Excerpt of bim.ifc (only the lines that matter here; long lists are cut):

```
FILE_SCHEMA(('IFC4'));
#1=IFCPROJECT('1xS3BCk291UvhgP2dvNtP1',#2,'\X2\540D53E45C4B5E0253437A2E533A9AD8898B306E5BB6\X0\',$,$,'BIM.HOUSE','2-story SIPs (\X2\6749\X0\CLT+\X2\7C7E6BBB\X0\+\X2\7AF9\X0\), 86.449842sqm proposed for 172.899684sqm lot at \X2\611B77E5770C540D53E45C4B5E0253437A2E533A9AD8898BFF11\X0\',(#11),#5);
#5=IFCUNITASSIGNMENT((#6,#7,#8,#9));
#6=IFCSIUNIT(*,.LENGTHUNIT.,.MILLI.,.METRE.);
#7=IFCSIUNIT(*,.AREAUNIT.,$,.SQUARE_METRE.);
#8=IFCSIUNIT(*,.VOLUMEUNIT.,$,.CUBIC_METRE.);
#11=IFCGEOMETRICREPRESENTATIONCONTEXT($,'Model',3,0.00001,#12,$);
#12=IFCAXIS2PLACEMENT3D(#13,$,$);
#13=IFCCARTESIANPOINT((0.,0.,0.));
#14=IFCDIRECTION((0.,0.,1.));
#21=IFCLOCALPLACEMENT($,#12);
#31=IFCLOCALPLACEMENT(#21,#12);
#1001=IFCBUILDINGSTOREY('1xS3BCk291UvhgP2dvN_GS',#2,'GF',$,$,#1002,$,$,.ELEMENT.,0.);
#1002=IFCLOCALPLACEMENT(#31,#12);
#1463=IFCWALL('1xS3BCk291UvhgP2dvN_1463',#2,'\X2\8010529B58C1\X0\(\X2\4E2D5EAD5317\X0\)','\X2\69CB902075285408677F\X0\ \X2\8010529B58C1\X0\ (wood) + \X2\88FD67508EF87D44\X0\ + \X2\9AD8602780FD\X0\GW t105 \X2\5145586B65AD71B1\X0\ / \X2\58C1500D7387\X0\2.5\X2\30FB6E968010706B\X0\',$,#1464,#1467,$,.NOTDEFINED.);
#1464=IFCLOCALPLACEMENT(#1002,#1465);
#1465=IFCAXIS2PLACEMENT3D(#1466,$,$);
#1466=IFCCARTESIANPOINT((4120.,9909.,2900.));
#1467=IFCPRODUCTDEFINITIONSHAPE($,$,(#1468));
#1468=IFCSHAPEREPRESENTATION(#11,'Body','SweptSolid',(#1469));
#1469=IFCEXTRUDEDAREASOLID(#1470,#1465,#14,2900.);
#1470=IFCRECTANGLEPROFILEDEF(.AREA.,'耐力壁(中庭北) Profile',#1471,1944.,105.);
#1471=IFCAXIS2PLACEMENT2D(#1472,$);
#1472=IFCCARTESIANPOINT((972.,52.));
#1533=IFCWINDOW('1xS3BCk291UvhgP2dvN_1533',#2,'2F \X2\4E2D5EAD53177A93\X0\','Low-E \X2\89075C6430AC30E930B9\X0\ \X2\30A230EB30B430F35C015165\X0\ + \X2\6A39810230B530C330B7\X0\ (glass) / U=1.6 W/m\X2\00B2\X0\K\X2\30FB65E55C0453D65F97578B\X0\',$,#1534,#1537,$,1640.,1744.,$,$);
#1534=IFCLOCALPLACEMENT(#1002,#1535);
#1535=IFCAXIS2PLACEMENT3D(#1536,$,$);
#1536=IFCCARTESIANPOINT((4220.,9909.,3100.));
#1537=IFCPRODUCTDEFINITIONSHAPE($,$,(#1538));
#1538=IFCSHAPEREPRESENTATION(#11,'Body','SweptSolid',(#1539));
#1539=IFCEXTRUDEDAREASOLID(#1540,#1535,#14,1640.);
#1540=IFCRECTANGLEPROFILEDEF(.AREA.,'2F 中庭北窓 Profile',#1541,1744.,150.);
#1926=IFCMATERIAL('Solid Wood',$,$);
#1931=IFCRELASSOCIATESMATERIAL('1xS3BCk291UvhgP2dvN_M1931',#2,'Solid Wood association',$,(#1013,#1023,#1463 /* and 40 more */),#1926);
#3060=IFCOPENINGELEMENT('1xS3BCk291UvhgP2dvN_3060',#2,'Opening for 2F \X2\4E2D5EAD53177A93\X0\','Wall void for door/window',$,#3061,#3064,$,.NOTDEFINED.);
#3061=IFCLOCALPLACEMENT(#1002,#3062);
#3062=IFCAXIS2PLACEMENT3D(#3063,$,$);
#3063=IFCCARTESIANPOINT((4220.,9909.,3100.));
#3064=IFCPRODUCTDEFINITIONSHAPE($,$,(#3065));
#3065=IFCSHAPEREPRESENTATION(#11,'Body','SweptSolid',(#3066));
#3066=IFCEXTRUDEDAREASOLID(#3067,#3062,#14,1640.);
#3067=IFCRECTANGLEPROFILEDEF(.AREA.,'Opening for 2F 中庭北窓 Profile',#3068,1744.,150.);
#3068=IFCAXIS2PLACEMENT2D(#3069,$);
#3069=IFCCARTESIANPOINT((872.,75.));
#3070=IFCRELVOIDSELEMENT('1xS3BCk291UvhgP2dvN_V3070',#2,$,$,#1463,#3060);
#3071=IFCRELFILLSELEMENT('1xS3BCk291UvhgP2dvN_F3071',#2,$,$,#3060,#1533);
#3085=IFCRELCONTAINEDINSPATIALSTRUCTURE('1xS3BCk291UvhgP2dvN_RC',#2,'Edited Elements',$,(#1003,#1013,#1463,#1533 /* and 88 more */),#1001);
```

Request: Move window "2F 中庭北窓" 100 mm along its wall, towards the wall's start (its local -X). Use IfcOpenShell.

```python
import ifcopenshell
import ifcopenshell.api.geometry
import ifcopenshell.util.placement

model = ifcopenshell.open("bim.ifc")

window = model.by_guid("1xS3BCk291UvhgP2dvN_1533")
opening = window.FillsVoids[0].RelatingOpeningElement
wall = opening.VoidsElements[0].RelatingBuildingElement

wall_matrix = ifcopenshell.util.placement.get_local_placement(wall.ObjectPlacement)
shift = wall_matrix[:3, 0] * -100.0
before = ifcopenshell.util.placement.get_local_placement(window.ObjectPlacement)[:3, 3].copy()

# The window is not placed relative to its opening, so move both.
for product in (opening, window):
    matrix = ifcopenshell.util.placement.get_local_placement(product.ObjectPlacement)
    matrix[:3, 3] += shift
    ifcopenshell.api.geometry.edit_object_placement(model, product=product, matrix=matrix, is_si=False)

after = ifcopenshell.util.placement.get_local_placement(window.ObjectPlacement)[:3, 3]
print("window moved by", (after - before).round(3) + 0.0)

model.write("bim-out.ifc")
```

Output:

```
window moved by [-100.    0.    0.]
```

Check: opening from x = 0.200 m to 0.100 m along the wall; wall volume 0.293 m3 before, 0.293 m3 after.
